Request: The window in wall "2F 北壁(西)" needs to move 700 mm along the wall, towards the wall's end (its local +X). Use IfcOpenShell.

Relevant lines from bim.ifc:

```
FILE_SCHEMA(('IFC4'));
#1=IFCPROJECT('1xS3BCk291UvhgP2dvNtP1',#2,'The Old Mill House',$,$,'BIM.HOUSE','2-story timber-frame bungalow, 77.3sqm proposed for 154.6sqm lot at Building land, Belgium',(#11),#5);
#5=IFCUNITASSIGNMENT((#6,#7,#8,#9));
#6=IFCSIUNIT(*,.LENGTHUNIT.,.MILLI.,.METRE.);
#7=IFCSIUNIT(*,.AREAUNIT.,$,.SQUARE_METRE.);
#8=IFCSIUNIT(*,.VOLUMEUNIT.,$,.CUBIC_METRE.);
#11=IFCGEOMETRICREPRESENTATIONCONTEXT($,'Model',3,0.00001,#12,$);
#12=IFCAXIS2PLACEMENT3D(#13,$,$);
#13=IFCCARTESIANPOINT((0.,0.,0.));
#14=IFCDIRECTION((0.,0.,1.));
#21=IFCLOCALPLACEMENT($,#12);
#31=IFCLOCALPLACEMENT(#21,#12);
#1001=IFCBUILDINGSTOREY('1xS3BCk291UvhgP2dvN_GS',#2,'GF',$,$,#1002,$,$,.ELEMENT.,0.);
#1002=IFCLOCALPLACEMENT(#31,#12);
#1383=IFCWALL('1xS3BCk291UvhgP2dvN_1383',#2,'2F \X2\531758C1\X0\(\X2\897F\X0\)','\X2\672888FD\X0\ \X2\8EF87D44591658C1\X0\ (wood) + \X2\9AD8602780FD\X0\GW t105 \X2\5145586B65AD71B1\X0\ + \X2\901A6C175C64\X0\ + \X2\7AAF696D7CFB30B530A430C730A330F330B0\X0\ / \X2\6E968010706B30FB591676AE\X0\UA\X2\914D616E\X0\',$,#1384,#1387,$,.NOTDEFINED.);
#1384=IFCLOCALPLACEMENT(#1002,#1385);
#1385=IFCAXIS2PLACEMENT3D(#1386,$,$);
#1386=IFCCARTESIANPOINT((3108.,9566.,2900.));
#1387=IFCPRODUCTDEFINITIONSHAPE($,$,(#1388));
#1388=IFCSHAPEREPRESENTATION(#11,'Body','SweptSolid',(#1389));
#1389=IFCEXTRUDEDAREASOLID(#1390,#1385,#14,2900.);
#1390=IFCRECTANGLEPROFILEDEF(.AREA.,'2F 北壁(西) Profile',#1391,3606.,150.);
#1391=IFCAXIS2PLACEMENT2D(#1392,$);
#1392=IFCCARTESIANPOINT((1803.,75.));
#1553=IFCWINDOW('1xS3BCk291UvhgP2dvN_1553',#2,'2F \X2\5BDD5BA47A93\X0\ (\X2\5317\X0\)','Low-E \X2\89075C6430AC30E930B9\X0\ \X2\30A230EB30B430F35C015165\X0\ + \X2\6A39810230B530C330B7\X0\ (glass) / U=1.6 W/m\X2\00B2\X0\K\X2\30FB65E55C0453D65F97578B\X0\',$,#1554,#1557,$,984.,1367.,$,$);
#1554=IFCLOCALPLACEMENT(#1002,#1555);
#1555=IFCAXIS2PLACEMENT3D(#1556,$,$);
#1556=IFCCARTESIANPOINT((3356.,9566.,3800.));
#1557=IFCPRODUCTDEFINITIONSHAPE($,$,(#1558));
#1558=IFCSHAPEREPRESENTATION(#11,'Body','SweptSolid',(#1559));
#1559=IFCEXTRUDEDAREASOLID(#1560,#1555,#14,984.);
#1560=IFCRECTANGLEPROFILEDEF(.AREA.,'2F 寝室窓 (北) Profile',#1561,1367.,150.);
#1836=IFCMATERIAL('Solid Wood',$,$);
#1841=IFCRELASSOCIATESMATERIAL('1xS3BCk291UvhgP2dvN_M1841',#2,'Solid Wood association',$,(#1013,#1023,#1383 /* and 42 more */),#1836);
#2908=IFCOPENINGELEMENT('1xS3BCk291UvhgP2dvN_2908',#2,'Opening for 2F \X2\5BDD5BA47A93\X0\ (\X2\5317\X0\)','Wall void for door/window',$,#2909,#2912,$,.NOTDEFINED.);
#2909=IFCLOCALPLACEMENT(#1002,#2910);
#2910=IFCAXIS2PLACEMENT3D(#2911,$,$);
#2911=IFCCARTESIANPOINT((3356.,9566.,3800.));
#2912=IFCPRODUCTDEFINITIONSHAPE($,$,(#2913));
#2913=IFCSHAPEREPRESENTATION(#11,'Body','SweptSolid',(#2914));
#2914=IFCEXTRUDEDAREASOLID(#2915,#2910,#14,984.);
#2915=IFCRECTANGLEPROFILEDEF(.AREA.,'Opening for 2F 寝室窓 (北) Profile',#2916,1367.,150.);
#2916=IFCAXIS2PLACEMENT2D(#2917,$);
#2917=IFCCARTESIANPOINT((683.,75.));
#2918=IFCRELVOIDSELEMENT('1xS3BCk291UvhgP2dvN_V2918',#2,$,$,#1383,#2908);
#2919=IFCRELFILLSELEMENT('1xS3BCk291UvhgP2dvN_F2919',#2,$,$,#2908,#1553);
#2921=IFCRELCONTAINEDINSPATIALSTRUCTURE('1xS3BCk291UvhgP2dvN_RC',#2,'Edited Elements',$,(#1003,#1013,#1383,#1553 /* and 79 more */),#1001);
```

```python
import ifcopenshell
import ifcopenshell.api.geometry
import ifcopenshell.util.placement
import ifcopenshell.util.unit

model = ifcopenshell.open("bim.ifc")
unit_scale = ifcopenshell.util.unit.calculate_unit_scale(model)

window = model.by_guid("1xS3BCk291UvhgP2dvN_1553")
opening = window.FillsVoids[0].RelatingOpeningElement
wall = opening.VoidsElements[0].RelatingBuildingElement

wall_matrix = ifcopenshell.util.placement.get_local_placement(wall.ObjectPlacement)
shift = wall_matrix[:3, 0] * 0.7 / unit_scale
before = ifcopenshell.util.placement.get_local_placement(window.ObjectPlacement)[:3, 3].copy()

# The window is not placed relative to its opening, so move both.
for product in (opening, window):
    matrix = ifcopenshell.util.placement.get_local_placement(product.ObjectPlacement)
    matrix[:3, 3] += shift
    ifcopenshell.api.geometry.edit_object_placement(model, product=product, matrix=matrix, is_si=False)

after = ifcopenshell.util.placement.get_local_placement(window.ObjectPlacement)[:3, 3]
print("window moved by", (after - before).round(3) + 0.0)

model.write("bim_rev.ifc")
```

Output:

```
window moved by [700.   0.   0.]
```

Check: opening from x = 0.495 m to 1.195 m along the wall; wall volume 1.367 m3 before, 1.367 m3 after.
